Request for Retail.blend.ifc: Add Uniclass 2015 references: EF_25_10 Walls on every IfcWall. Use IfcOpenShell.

First a look at what the model holds.

```python
import ifcopenshell

model = ifcopenshell.open("Retail.blend.ifc")
print(model.schema)
print("classifications:", [c.Name for c in model.by_type("IfcClassification")])
for ifc_class in ("IfcDoor", "IfcRoof", "IfcStair", "IfcWall", "IfcWindow"):
    print(ifc_class, len(model.by_type(ifc_class)))
```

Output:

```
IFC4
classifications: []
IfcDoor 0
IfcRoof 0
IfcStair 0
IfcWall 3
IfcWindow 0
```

```python
import ifcopenshell
import ifcopenshell.api.classification

model = ifcopenshell.open("Retail.blend.ifc")

system = ifcopenshell.api.classification.add_classification(model, classification="Uniclass 2015")

codes = {
    "IfcWall": ("EF_25_10", "Walls"),
}
for ifc_class, (code, name) in codes.items():
    products = model.by_type(ifc_class)
    ifcopenshell.api.classification.add_reference(
        model, products=products, classification=system, identification=code, name=name
    )
    print(code, len(products))

model.write("Retail.blend_v2.ifc")
```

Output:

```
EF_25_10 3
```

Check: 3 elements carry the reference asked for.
